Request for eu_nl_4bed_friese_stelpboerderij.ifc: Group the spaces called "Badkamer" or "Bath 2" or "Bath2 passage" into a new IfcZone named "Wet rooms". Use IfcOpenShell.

First a look at what the model holds.

```python
import ifcopenshell

model = ifcopenshell.open("eu_nl_4bed_friese_stelpboerderij.ifc")
print(model.schema)
seen = {}
for space in model.by_type("IfcSpace"):
    seen[space.LongName] = seen.get(space.LongName, 0) + 1
for name, count in sorted(seen.items(), key=str):
    print(count, "x", name)
print("zones:", [z.Name for z in model.by_type("IfcZone")][:20])
```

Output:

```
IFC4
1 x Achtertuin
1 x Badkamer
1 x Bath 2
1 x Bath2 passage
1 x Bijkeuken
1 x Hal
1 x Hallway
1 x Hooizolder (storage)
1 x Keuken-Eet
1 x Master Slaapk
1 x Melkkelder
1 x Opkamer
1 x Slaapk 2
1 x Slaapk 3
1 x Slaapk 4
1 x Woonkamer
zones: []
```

```python
import ifcopenshell
import ifcopenshell.api.group
import ifcopenshell.api.root

model = ifcopenshell.open("eu_nl_4bed_friese_stelpboerderij.ifc")

names = {"Badkamer", "Bath 2", "Bath2 passage"}
spaces = [s for s in model.by_type("IfcSpace") if s.LongName in names]

zone = ifcopenshell.api.root.create_entity(model, ifc_class="IfcZone", name="Wet rooms")
ifcopenshell.api.group.assign_group(model, products=spaces, group=zone)
print(len(spaces), "spaces in", zone.Name)

model.write("eu_nl_4bed_friese_stelpboerderij_rev.ifc")
```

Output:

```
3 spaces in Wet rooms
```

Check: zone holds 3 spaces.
